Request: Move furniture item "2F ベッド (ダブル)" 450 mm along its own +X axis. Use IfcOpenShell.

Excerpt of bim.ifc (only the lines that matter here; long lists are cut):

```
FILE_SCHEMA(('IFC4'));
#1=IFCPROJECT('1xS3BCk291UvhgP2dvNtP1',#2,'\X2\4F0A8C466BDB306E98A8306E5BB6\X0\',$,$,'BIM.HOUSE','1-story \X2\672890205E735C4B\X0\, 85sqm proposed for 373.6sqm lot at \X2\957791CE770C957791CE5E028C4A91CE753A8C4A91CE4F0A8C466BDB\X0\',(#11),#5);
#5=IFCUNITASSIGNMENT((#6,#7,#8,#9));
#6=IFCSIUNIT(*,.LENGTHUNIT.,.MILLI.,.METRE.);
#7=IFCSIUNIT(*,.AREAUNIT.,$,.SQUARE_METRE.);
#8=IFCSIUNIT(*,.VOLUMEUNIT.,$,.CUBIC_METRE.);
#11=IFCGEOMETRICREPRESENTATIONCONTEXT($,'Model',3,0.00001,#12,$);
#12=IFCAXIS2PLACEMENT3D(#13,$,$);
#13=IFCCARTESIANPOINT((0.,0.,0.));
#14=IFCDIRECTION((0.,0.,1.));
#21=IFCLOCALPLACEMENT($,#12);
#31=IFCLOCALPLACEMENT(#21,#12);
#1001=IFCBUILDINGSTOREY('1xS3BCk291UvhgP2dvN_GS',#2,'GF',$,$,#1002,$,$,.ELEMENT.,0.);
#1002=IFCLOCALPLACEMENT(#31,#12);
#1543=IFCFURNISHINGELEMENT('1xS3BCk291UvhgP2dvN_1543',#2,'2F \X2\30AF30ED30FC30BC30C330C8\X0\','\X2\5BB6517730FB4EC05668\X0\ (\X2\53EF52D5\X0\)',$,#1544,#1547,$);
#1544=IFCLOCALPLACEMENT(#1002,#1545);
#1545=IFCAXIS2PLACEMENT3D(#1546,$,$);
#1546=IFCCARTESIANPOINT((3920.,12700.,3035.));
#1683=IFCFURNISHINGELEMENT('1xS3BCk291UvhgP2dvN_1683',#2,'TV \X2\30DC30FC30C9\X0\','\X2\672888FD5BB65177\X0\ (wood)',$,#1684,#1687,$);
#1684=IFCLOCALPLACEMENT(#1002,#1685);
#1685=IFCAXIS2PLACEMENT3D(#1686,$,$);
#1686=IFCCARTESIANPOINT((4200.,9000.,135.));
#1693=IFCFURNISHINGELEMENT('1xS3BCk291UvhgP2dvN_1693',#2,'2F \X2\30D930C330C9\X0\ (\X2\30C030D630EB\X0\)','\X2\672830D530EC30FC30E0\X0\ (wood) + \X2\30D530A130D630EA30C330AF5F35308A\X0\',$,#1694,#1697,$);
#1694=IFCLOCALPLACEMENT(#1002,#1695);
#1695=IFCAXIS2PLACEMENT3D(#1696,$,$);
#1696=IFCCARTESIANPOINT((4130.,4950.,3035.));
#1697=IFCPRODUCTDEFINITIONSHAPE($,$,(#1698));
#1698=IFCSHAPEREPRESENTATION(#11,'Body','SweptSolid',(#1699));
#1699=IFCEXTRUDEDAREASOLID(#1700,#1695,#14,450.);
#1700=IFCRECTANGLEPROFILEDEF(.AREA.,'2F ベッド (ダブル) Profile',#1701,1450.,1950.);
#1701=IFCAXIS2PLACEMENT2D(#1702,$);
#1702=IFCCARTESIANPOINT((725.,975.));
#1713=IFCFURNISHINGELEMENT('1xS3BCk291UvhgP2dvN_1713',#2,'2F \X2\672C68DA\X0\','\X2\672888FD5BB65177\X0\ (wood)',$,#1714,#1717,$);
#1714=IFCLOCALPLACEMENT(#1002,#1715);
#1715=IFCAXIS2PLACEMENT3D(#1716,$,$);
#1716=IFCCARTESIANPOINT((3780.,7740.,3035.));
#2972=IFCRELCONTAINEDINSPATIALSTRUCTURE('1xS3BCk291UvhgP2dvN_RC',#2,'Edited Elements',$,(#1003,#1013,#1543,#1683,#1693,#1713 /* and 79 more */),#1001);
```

```python
import ifcopenshell
import ifcopenshell.api.geometry
import ifcopenshell.util.placement

model = ifcopenshell.open("bim.ifc")

item = model.by_guid("1xS3BCk291UvhgP2dvN_1693")
matrix = ifcopenshell.util.placement.get_local_placement(item.ObjectPlacement)
matrix[:3, 3] += matrix[:3, 0] * 450.0
ifcopenshell.api.geometry.edit_object_placement(model, product=item, matrix=matrix, is_si=False)

print(ifcopenshell.util.placement.get_local_placement(item.ObjectPlacement).round(3) + 0.0)

model.write("bim_rev.ifc")
```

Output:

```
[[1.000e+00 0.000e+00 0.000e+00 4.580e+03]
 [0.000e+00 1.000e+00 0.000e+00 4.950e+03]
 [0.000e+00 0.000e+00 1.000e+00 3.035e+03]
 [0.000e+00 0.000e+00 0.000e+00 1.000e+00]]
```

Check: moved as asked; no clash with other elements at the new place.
